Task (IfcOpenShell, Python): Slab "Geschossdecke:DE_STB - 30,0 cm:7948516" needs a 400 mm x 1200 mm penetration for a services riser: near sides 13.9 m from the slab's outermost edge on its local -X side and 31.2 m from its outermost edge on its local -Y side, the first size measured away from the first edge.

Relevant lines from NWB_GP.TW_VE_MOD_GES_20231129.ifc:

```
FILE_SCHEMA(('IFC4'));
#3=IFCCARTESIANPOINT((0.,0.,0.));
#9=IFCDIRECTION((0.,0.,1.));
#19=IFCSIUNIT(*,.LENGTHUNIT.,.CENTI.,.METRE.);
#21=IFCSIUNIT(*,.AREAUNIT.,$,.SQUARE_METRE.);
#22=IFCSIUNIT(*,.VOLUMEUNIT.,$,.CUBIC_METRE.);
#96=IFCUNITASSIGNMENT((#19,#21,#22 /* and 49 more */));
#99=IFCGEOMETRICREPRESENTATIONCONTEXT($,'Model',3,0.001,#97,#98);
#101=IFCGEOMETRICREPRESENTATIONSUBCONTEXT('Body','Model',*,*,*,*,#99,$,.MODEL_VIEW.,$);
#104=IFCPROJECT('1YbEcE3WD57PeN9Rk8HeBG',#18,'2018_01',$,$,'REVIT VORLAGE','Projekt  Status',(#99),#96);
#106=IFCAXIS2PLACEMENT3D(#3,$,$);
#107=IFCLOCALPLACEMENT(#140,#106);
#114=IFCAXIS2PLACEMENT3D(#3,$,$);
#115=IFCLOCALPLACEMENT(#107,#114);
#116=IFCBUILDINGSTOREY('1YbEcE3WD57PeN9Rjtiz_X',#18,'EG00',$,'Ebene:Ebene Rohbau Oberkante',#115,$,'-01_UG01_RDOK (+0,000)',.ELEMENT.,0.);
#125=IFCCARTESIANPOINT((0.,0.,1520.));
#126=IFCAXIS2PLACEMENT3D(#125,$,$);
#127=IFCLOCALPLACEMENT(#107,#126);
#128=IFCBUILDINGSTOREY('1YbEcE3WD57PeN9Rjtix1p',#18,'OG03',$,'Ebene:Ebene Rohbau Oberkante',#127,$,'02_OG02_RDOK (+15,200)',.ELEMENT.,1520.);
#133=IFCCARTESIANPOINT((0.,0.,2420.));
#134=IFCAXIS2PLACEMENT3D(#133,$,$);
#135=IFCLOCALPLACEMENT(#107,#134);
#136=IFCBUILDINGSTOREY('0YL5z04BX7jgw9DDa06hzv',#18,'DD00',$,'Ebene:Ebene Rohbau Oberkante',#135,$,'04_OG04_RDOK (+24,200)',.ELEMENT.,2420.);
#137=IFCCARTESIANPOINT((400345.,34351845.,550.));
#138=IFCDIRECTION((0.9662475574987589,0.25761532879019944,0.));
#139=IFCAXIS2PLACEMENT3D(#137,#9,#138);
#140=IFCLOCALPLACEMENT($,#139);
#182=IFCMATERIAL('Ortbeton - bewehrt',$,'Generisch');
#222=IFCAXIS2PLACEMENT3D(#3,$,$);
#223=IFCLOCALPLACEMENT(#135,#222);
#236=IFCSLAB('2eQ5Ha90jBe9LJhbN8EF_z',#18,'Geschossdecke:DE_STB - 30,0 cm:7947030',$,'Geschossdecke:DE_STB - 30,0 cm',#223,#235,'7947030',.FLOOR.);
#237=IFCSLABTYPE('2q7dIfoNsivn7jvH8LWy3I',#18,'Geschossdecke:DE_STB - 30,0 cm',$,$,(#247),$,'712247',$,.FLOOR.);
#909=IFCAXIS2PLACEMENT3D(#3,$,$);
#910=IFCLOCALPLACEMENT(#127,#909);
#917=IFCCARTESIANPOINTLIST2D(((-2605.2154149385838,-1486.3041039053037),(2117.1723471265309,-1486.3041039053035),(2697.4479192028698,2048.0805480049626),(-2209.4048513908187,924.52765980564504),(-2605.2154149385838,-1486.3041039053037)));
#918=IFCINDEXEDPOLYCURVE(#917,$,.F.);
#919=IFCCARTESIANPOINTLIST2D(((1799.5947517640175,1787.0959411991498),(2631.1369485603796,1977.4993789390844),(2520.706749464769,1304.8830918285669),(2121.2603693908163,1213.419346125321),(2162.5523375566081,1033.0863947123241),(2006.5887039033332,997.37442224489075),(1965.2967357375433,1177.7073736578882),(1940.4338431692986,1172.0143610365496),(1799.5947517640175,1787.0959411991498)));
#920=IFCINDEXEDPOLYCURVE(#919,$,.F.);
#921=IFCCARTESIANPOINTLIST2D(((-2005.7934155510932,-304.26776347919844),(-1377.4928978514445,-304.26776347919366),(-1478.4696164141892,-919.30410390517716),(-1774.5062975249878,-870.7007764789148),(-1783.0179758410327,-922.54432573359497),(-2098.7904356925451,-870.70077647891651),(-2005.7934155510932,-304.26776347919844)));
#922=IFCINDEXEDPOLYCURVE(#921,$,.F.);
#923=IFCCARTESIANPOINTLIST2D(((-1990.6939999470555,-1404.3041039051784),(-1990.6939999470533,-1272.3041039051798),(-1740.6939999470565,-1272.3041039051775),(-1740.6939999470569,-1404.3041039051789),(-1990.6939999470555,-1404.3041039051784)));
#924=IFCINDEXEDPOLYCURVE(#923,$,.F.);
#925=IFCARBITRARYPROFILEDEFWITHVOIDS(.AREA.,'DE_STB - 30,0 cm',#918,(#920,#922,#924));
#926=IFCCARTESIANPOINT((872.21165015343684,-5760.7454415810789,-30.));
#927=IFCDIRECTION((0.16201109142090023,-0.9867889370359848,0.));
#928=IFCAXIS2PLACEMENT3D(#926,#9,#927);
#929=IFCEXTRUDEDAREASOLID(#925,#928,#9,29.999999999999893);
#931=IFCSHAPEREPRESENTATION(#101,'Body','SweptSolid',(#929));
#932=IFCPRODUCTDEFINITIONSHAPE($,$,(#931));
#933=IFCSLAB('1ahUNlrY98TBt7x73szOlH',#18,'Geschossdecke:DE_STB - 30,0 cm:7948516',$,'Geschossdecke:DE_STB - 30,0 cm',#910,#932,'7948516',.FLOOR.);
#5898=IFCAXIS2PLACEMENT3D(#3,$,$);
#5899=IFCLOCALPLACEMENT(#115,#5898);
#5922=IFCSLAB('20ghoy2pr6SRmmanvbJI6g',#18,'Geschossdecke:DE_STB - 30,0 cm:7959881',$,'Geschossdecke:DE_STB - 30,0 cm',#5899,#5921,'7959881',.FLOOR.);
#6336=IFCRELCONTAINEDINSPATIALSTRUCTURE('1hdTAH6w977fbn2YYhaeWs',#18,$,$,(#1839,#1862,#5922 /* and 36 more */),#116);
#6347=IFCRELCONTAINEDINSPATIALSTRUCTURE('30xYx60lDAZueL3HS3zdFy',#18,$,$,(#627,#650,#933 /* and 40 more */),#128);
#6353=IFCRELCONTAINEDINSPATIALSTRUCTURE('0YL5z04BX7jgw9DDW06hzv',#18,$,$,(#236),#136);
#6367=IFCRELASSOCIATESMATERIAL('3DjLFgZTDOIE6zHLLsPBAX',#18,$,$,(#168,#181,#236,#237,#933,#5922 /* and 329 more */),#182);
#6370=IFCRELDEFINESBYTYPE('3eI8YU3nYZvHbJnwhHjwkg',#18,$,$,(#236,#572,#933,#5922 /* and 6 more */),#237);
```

```python
import numpy as np
import ifcopenshell
import ifcopenshell.api.feature
import ifcopenshell.api.geometry
import ifcopenshell.api.root
import ifcopenshell.geom
import ifcopenshell.util.placement
import ifcopenshell.util.representation
import ifcopenshell.util.shape
import ifcopenshell.util.unit

model = ifcopenshell.open("NWB_GP.TW_VE_MOD_GES_20231129.ifc")
unit_scale = ifcopenshell.util.unit.calculate_unit_scale(model)
settings = ifcopenshell.geom.settings()


def volume(element):
    """Net volume in cubic metres, openings subtracted."""
    shape = ifcopenshell.geom.create_shape(settings, element)
    return ifcopenshell.util.shape.get_volume(shape.geometry)


slab = model.by_id(933)
before = volume(slab)

# Extent in the slab's own axes, in metres. The edges named are its -X and -Y sides.
slab_shape = ifcopenshell.geom.create_shape(settings, slab)
vertices = ifcopenshell.util.shape.get_vertices(slab_shape.geometry)
x_min, y_min, bottom = vertices.min(axis=0)
top = vertices[:, 2].max()

opening = ifcopenshell.api.root.create_entity(model, ifc_class="IfcOpeningElement", name="Services riser opening", predefined_type="OPENING")
context = ifcopenshell.util.representation.get_context(model, "Model", "Body", "MODEL_VIEW")
width, depth = 0.4, 1.2
outline = [(0.0, 0.0), (width, 0.0), (width, depth), (0.0, depth), (0.0, 0.0)]
# Overshoot both faces by 50 mm so the cut is clean.
shape = ifcopenshell.api.geometry.add_slab_representation(
    model, context=context, depth=top - bottom + 0.1, polyline=outline
)
ifcopenshell.api.geometry.assign_representation(model, product=opening, representation=shape)

matrix = ifcopenshell.util.placement.get_local_placement(slab.ObjectPlacement)
matrix[:, 3] = matrix @ np.append(np.array([x_min + 13.9, y_min + 31.2, bottom - 0.05]) / unit_scale, 1.0)
ifcopenshell.api.geometry.edit_object_placement(model, product=opening, matrix=matrix, is_si=False)
ifcopenshell.api.feature.add_feature(model, feature=opening, element=slab)

after = volume(slab)

print(f"slab volume {before:.3f} -> {after:.3f} m3")

model.write("NWB_GP.TW_VE_MOD_GES_20231129-out.ifc")
```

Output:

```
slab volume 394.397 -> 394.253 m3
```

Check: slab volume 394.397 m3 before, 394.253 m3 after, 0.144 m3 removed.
